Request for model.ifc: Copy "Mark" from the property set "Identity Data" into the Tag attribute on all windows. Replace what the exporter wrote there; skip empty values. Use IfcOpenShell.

First a look at what the model holds.

```python
import ifcopenshell
import ifcopenshell.util.element

model = ifcopenshell.open("model.ifc")
print(model.schema)
windows = model.by_type("IfcWindow")
print(len(windows), "windows")
for e in windows[:8]:
    source = ifcopenshell.util.element.get_pset(e, "Identity Data", "Mark")
    target = e.Tag
    print(e.id(), repr(source), repr(target), sep=" | ")
```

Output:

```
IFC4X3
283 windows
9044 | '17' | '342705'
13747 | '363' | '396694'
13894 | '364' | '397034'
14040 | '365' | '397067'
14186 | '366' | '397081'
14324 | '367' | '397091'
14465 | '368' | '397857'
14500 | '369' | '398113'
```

```python
import ifcopenshell
import ifcopenshell.util.element

model = ifcopenshell.open("model.ifc")

count = 0
for e in model.by_type("IfcWindow"):
    value = ifcopenshell.util.element.get_pset(e, "Identity Data", "Mark")
    current = e.Tag
    if not value or not value.strip() or current == value:
        continue
    e.Tag = value
    count += 1

print(count, "windows updated")

model.write("model_v2.ifc")
```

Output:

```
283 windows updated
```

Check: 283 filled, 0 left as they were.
